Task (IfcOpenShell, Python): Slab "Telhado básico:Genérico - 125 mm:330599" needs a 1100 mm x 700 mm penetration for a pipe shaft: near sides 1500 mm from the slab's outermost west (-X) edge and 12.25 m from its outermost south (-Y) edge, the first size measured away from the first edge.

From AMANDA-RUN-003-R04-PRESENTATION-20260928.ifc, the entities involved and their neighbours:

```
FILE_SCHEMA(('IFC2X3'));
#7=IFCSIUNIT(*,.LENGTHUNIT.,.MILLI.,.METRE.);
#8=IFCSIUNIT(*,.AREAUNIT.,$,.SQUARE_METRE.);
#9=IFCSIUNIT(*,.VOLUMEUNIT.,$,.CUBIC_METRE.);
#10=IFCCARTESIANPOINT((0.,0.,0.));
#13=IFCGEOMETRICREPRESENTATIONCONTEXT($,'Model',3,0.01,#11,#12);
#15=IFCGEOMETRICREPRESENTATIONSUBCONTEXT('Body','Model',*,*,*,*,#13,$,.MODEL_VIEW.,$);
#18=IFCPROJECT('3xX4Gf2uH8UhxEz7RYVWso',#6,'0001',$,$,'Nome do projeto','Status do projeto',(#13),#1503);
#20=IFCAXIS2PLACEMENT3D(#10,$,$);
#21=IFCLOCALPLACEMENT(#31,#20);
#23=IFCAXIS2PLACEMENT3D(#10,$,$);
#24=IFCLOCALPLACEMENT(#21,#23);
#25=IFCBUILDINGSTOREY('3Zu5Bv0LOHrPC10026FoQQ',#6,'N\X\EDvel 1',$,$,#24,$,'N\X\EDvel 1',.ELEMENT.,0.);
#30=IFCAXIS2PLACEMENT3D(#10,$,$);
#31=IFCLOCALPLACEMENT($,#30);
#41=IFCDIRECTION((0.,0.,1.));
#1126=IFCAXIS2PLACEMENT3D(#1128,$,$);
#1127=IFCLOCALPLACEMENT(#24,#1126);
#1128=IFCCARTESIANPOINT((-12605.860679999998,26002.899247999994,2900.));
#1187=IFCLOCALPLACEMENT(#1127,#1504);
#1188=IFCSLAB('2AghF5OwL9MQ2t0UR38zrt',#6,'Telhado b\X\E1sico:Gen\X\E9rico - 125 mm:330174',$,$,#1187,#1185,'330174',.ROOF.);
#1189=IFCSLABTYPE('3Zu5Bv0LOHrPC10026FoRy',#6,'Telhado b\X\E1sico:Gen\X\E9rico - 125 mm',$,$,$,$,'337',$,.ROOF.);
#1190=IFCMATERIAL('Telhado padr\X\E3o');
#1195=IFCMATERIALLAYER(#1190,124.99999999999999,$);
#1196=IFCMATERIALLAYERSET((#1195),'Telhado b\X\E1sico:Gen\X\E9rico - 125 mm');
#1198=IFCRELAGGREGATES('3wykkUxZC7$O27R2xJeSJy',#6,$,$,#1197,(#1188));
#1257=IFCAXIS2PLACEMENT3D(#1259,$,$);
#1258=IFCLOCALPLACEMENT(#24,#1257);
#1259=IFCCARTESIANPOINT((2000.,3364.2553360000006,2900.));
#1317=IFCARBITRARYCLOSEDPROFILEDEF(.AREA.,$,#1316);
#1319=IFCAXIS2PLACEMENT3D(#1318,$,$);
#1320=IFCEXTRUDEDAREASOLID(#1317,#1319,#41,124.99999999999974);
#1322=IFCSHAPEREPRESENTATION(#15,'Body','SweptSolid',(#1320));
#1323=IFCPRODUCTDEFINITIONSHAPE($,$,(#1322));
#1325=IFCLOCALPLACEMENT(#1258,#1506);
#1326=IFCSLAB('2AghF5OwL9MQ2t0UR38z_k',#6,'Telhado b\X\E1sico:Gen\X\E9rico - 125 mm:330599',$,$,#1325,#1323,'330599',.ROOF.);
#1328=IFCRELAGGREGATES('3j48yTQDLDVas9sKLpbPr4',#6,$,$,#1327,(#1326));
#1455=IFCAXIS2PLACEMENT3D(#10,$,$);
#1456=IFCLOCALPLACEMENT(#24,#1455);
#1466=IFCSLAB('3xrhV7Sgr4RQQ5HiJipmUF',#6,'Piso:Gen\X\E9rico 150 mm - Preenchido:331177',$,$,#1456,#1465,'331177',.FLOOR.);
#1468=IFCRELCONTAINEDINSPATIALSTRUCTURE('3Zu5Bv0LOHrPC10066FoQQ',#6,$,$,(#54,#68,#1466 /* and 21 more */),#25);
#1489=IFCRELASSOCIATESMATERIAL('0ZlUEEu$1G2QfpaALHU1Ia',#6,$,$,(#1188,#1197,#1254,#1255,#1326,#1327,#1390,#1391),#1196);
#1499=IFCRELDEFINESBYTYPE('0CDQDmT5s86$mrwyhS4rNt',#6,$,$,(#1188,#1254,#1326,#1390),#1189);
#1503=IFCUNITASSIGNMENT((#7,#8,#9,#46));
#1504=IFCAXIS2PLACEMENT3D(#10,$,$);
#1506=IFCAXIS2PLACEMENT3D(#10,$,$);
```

```python
import numpy as np
import ifcopenshell
import ifcopenshell.api.feature
import ifcopenshell.api.geometry
import ifcopenshell.api.root
import ifcopenshell.geom
import ifcopenshell.util.placement
import ifcopenshell.util.representation
import ifcopenshell.util.shape
import ifcopenshell.util.unit

model = ifcopenshell.open("AMANDA-RUN-003-R04-PRESENTATION-20260928.ifc")
unit_scale = ifcopenshell.util.unit.calculate_unit_scale(model)
settings = ifcopenshell.geom.settings()


def volume(element):
    """Net volume in cubic metres, openings subtracted."""
    shape = ifcopenshell.geom.create_shape(settings, element)
    return ifcopenshell.util.shape.get_volume(shape.geometry)


slab = model.by_guid("2AghF5OwL9MQ2t0UR38z_k")
before = volume(slab)

# Extent in the slab's own axes, in metres. The edges named are its -X and -Y sides.
slab_shape = ifcopenshell.geom.create_shape(settings, slab)
vertices = ifcopenshell.util.shape.get_vertices(slab_shape.geometry)
x_min, y_min, bottom = vertices.min(axis=0)
top = vertices[:, 2].max()

opening = ifcopenshell.api.root.create_entity(model, ifc_class="IfcOpeningElement", name="Pipe shaft opening")
context = ifcopenshell.util.representation.get_context(model, "Model", "Body", "MODEL_VIEW")
width, depth = 1.1, 0.7
outline = [(0.0, 0.0), (width, 0.0), (width, depth), (0.0, depth), (0.0, 0.0)]
# Overshoot both faces by 50 mm so the cut is clean.
shape = ifcopenshell.api.geometry.add_slab_representation(
    model, context=context, depth=top - bottom + 0.1, polyline=outline
)
ifcopenshell.api.geometry.assign_representation(model, product=opening, representation=shape)

matrix = ifcopenshell.util.placement.get_local_placement(slab.ObjectPlacement)
matrix[:, 3] = matrix @ np.append(np.array([x_min + 1.5, y_min + 12.25, bottom - 0.05]) / unit_scale, 1.0)
ifcopenshell.api.geometry.edit_object_placement(model, product=opening, matrix=matrix, is_si=False)
ifcopenshell.api.feature.add_feature(model, feature=opening, element=slab)

after = volume(slab)

print(f"slab volume {before:.3f} -> {after:.3f} m3")

model.write("AMANDA-RUN-003-R04-PRESENTATION-20260928_edited.ifc")
```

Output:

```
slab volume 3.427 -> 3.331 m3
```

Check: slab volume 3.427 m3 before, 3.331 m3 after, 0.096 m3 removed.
